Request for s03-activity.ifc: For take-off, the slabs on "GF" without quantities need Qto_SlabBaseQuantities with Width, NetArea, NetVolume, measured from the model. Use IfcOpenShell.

First a look at what the model holds.

```python
import ifcopenshell
import ifcopenshell.util.element
import ifcopenshell.util.unit

model = ifcopenshell.open("s03-activity.ifc")
print(model.schema)
for unit_type in ("LENGTHUNIT", "AREAUNIT", "VOLUMEUNIT"):
    print(unit_type, ifcopenshell.util.unit.calculate_unit_scale(model, unit_type))
storey = next(s for s in model.by_type("IfcBuildingStorey") if s.Name == "GF")
slabs = [e for e in ifcopenshell.util.element.get_decomposition(storey) if e.is_a("IfcSlab")]
for e in sorted(slabs, key=lambda e: e.id()):
    print(e.id(), e.is_a(), e.Name, list(ifcopenshell.util.element.get_psets(e, qtos_only=True)), sep=" | ")
```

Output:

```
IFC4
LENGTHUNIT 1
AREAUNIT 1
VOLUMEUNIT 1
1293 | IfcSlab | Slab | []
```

```python
import ifcopenshell
import ifcopenshell.api.pset
import ifcopenshell.geom
import ifcopenshell.util.element
import ifcopenshell.util.shape
import ifcopenshell.util.unit

model = ifcopenshell.open("s03-activity.ifc")
unit_scale = ifcopenshell.util.unit.calculate_unit_scale(model)
area_scale = ifcopenshell.util.unit.calculate_unit_scale(model, "AREAUNIT")
volume_scale = ifcopenshell.util.unit.calculate_unit_scale(model, "VOLUMEUNIT")
settings = ifcopenshell.geom.settings()

storey = next(s for s in model.by_type("IfcBuildingStorey") if s.Name == "GF")
slabs = [e for e in ifcopenshell.util.element.get_decomposition(storey) if e.is_a("IfcSlab")]

for e in sorted(slabs, key=lambda e: e.id()):
    if ifcopenshell.util.element.get_psets(e, qtos_only=True, should_inherit=False):
        continue
    # Geometry comes back in metres, in the element's own axes.
    shape = ifcopenshell.geom.create_shape(settings, e)
    values = {
        "Width": ifcopenshell.util.shape.get_z(shape.geometry) / unit_scale,
        "NetArea": ifcopenshell.util.shape.get_footprint_area(shape.geometry) / area_scale,
        "NetVolume": ifcopenshell.util.shape.get_volume(shape.geometry) / volume_scale,
    }
    qto = ifcopenshell.api.pset.add_qto(model, product=e, name="Qto_SlabBaseQuantities")
    ifcopenshell.api.pset.edit_qto(model, qto=qto, properties=values)
    print(e.id(), {k: round(v, 3) for k, v in values.items()})

model.write("s03-activity_edited.ifc")
```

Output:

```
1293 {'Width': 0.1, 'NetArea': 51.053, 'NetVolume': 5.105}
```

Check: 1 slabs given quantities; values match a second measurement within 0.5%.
